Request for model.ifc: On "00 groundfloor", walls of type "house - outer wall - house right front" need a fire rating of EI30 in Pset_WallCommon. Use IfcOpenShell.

First a look at what the model holds.

```python
import ifcopenshell
import ifcopenshell.util.element

model = ifcopenshell.open("model.ifc")
print(model.schema)
storey = next(s for s in model.by_type("IfcBuildingStorey") if s.Name == "00 groundfloor")
walls = [e for e in ifcopenshell.util.element.get_decomposition(storey) if e.is_a("IfcWall")]
seen = {}
for e in walls:
    element_type = ifcopenshell.util.element.get_type(e)
    key = (element_type.Name if element_type != e and element_type else None, ifcopenshell.util.element.get_pset(e, "Pset_WallCommon", "FireRating"))
    seen[key] = seen.get(key, 0) + 1
for (name, value), count in sorted(seen.items(), key=str):
    print(count, "x", name, "|", value)
```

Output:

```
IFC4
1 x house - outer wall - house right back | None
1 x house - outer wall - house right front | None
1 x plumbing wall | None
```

```python
import ifcopenshell
import ifcopenshell.api.pset
import ifcopenshell.util.element

model = ifcopenshell.open("model.ifc")

storey = next(s for s in model.by_type("IfcBuildingStorey") if s.Name == "00 groundfloor")
walls = [e for e in ifcopenshell.util.element.get_decomposition(storey) if e.is_a("IfcWall")]

count = 0
for e in walls:
    element_type = ifcopenshell.util.element.get_type(e)
    if element_type in (None, e) or element_type.Name != "house - outer wall - house right front":
        continue
    # add_pset returns the element's existing set when there is one.
    pset = ifcopenshell.api.pset.add_pset(model, product=e, name="Pset_WallCommon")
    ifcopenshell.api.pset.edit_pset(model, pset=pset, properties={"FireRating": "EI30"})
    count += 1

print(count, "walls updated")

model.write("model_v2.ifc")
```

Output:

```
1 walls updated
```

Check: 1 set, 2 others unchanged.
